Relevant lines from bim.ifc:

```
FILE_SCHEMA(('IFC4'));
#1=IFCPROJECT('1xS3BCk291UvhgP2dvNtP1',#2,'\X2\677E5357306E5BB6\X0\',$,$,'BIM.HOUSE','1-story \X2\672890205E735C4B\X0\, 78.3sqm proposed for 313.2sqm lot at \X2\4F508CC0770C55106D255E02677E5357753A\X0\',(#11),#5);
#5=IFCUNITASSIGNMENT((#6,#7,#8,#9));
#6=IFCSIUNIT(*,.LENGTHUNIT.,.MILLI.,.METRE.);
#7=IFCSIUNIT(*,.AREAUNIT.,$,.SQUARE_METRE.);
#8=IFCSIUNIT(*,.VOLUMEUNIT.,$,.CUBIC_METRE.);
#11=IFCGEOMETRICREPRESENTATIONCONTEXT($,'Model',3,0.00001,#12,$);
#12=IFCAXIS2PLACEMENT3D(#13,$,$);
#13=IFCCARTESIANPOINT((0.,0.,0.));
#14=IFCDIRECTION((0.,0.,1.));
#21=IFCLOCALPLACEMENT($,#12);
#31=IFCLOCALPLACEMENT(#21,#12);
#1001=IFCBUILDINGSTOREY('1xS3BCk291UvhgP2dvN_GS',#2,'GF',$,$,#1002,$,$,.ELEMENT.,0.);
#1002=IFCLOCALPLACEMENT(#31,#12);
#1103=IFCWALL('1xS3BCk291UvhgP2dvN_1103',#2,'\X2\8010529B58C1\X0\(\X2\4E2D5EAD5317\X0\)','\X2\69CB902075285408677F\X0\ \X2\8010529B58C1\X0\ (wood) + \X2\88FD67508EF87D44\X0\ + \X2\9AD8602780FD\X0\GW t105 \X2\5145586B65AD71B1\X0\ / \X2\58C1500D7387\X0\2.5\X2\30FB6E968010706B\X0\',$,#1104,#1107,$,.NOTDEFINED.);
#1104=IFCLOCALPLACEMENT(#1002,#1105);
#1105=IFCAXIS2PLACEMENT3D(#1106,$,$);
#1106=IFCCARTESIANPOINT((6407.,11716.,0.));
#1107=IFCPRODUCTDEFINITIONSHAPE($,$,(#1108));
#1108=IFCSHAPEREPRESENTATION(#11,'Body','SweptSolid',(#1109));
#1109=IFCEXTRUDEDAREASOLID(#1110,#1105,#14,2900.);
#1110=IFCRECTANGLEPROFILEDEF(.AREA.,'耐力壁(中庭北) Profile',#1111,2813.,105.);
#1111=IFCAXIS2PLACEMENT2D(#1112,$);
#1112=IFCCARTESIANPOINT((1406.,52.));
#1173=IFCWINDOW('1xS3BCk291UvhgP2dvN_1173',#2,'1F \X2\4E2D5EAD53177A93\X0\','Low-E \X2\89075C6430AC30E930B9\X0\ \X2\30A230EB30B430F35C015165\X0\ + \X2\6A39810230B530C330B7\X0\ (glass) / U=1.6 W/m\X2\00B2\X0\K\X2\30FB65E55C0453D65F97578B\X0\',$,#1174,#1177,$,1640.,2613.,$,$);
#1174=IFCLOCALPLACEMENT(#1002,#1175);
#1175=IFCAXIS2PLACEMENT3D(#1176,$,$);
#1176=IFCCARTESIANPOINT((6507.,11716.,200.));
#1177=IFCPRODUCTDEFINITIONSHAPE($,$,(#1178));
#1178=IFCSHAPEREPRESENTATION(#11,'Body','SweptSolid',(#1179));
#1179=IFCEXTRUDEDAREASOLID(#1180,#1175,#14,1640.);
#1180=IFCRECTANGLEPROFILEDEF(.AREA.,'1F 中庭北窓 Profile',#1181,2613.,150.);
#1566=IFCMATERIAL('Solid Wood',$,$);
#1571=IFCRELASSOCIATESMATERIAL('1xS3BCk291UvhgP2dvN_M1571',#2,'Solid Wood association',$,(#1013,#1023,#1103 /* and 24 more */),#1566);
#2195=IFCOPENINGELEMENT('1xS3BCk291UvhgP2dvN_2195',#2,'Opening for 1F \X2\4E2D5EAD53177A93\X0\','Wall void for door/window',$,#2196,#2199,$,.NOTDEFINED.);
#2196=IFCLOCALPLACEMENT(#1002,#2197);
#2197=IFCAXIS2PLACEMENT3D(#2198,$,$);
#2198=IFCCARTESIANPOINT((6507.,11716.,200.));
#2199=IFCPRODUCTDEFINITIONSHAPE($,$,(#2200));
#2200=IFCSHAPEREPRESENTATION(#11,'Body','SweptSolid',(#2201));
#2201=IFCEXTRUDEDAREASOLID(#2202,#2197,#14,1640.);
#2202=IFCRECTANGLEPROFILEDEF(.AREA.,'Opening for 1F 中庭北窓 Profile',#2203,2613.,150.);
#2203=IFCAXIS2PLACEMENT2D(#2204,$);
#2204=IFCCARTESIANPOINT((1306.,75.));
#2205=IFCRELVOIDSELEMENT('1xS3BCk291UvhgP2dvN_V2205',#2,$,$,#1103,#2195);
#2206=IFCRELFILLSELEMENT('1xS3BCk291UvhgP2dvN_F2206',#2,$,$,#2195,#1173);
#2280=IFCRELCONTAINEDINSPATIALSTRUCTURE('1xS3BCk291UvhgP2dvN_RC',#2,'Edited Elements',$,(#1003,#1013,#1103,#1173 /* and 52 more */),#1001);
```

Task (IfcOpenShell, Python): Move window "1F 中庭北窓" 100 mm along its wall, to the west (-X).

```python
import ifcopenshell
import ifcopenshell.api.geometry
import ifcopenshell.util.placement
import ifcopenshell.util.unit

model = ifcopenshell.open("bim.ifc")
unit_scale = ifcopenshell.util.unit.calculate_unit_scale(model)

window = model.by_guid("1xS3BCk291UvhgP2dvN_1173")
opening = window.FillsVoids[0].RelatingOpeningElement
wall = opening.VoidsElements[0].RelatingBuildingElement

wall_matrix = ifcopenshell.util.placement.get_local_placement(wall.ObjectPlacement)
shift = wall_matrix[:3, 0] * -0.1 / unit_scale
before = ifcopenshell.util.placement.get_local_placement(window.ObjectPlacement)[:3, 3].copy()

# The window is not placed relative to its opening, so move both.
for product in (opening, window):
    matrix = ifcopenshell.util.placement.get_local_placement(product.ObjectPlacement)
    matrix[:3, 3] += shift
    ifcopenshell.api.geometry.edit_object_placement(model, product=product, matrix=matrix, is_si=False)

after = ifcopenshell.util.placement.get_local_placement(window.ObjectPlacement)[:3, 3]
print("window moved by", (after - before).round(3) + 0.0)

model.write("bim_edited.ifc")
```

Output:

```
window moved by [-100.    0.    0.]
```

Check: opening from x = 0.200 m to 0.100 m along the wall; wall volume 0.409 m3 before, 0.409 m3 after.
